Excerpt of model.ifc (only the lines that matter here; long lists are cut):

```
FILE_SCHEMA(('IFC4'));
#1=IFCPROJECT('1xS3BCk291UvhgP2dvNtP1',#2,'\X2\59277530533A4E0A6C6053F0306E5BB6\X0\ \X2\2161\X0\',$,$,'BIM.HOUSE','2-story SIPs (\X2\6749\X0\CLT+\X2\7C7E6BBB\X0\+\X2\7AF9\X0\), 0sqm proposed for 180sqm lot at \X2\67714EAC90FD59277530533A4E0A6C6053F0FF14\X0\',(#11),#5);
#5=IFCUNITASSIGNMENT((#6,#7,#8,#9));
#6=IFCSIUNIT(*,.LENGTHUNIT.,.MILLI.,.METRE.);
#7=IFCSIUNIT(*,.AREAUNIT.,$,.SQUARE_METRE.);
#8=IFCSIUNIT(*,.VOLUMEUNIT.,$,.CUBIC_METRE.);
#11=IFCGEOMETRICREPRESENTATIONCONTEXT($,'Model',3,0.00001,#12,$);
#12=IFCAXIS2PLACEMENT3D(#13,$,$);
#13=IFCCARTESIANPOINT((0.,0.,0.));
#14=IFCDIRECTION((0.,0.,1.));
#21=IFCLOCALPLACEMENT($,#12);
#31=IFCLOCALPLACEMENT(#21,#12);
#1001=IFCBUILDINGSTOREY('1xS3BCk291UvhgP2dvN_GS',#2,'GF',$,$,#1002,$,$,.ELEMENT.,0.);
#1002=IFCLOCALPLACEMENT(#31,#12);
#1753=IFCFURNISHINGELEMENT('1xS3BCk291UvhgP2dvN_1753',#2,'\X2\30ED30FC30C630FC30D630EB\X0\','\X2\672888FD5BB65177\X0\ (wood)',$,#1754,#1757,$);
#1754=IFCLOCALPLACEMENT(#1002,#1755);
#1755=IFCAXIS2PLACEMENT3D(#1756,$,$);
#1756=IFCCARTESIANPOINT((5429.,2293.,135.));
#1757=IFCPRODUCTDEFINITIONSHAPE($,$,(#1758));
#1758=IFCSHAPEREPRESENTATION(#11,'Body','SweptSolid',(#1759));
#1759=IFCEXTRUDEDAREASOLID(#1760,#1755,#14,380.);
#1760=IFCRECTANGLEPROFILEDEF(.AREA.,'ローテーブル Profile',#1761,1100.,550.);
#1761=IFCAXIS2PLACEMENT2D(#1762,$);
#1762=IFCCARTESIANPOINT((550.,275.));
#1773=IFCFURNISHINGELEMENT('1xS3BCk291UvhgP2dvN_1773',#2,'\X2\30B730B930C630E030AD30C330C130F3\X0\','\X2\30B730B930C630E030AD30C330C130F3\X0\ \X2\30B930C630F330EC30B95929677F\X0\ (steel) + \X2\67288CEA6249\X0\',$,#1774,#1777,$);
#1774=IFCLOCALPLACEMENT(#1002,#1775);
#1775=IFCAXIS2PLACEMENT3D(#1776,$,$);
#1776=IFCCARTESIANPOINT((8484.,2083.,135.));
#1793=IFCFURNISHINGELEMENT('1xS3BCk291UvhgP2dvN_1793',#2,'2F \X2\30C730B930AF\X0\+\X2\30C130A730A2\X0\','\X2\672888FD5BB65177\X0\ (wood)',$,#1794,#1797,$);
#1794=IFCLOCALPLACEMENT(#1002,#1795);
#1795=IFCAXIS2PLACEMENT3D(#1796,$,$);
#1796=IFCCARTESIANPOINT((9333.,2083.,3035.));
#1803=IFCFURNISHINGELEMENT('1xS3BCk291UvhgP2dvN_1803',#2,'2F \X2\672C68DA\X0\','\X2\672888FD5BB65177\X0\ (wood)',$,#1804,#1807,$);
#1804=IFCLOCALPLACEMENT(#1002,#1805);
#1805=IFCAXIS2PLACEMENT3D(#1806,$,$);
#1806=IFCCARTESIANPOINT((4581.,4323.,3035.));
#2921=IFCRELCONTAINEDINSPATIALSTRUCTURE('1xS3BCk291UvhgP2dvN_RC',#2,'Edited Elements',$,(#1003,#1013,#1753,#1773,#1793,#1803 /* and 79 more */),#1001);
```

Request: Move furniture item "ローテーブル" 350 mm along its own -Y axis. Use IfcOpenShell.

```python
import ifcopenshell
import ifcopenshell.api.geometry
import ifcopenshell.util.placement
import ifcopenshell.util.unit

model = ifcopenshell.open("model.ifc")
unit_scale = ifcopenshell.util.unit.calculate_unit_scale(model)

item = model.by_guid("1xS3BCk291UvhgP2dvN_1753")
matrix = ifcopenshell.util.placement.get_local_placement(item.ObjectPlacement)
matrix[:3, 3] -= matrix[:3, 1] * 0.35 / unit_scale
ifcopenshell.api.geometry.edit_object_placement(model, product=item, matrix=matrix, is_si=False)

print(ifcopenshell.util.placement.get_local_placement(item.ObjectPlacement).round(3) + 0.0)

model.write("model_edited.ifc")
```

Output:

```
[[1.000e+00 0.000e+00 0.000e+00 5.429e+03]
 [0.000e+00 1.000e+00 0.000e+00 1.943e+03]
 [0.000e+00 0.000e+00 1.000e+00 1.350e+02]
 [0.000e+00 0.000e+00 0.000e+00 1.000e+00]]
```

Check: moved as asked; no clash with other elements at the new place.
